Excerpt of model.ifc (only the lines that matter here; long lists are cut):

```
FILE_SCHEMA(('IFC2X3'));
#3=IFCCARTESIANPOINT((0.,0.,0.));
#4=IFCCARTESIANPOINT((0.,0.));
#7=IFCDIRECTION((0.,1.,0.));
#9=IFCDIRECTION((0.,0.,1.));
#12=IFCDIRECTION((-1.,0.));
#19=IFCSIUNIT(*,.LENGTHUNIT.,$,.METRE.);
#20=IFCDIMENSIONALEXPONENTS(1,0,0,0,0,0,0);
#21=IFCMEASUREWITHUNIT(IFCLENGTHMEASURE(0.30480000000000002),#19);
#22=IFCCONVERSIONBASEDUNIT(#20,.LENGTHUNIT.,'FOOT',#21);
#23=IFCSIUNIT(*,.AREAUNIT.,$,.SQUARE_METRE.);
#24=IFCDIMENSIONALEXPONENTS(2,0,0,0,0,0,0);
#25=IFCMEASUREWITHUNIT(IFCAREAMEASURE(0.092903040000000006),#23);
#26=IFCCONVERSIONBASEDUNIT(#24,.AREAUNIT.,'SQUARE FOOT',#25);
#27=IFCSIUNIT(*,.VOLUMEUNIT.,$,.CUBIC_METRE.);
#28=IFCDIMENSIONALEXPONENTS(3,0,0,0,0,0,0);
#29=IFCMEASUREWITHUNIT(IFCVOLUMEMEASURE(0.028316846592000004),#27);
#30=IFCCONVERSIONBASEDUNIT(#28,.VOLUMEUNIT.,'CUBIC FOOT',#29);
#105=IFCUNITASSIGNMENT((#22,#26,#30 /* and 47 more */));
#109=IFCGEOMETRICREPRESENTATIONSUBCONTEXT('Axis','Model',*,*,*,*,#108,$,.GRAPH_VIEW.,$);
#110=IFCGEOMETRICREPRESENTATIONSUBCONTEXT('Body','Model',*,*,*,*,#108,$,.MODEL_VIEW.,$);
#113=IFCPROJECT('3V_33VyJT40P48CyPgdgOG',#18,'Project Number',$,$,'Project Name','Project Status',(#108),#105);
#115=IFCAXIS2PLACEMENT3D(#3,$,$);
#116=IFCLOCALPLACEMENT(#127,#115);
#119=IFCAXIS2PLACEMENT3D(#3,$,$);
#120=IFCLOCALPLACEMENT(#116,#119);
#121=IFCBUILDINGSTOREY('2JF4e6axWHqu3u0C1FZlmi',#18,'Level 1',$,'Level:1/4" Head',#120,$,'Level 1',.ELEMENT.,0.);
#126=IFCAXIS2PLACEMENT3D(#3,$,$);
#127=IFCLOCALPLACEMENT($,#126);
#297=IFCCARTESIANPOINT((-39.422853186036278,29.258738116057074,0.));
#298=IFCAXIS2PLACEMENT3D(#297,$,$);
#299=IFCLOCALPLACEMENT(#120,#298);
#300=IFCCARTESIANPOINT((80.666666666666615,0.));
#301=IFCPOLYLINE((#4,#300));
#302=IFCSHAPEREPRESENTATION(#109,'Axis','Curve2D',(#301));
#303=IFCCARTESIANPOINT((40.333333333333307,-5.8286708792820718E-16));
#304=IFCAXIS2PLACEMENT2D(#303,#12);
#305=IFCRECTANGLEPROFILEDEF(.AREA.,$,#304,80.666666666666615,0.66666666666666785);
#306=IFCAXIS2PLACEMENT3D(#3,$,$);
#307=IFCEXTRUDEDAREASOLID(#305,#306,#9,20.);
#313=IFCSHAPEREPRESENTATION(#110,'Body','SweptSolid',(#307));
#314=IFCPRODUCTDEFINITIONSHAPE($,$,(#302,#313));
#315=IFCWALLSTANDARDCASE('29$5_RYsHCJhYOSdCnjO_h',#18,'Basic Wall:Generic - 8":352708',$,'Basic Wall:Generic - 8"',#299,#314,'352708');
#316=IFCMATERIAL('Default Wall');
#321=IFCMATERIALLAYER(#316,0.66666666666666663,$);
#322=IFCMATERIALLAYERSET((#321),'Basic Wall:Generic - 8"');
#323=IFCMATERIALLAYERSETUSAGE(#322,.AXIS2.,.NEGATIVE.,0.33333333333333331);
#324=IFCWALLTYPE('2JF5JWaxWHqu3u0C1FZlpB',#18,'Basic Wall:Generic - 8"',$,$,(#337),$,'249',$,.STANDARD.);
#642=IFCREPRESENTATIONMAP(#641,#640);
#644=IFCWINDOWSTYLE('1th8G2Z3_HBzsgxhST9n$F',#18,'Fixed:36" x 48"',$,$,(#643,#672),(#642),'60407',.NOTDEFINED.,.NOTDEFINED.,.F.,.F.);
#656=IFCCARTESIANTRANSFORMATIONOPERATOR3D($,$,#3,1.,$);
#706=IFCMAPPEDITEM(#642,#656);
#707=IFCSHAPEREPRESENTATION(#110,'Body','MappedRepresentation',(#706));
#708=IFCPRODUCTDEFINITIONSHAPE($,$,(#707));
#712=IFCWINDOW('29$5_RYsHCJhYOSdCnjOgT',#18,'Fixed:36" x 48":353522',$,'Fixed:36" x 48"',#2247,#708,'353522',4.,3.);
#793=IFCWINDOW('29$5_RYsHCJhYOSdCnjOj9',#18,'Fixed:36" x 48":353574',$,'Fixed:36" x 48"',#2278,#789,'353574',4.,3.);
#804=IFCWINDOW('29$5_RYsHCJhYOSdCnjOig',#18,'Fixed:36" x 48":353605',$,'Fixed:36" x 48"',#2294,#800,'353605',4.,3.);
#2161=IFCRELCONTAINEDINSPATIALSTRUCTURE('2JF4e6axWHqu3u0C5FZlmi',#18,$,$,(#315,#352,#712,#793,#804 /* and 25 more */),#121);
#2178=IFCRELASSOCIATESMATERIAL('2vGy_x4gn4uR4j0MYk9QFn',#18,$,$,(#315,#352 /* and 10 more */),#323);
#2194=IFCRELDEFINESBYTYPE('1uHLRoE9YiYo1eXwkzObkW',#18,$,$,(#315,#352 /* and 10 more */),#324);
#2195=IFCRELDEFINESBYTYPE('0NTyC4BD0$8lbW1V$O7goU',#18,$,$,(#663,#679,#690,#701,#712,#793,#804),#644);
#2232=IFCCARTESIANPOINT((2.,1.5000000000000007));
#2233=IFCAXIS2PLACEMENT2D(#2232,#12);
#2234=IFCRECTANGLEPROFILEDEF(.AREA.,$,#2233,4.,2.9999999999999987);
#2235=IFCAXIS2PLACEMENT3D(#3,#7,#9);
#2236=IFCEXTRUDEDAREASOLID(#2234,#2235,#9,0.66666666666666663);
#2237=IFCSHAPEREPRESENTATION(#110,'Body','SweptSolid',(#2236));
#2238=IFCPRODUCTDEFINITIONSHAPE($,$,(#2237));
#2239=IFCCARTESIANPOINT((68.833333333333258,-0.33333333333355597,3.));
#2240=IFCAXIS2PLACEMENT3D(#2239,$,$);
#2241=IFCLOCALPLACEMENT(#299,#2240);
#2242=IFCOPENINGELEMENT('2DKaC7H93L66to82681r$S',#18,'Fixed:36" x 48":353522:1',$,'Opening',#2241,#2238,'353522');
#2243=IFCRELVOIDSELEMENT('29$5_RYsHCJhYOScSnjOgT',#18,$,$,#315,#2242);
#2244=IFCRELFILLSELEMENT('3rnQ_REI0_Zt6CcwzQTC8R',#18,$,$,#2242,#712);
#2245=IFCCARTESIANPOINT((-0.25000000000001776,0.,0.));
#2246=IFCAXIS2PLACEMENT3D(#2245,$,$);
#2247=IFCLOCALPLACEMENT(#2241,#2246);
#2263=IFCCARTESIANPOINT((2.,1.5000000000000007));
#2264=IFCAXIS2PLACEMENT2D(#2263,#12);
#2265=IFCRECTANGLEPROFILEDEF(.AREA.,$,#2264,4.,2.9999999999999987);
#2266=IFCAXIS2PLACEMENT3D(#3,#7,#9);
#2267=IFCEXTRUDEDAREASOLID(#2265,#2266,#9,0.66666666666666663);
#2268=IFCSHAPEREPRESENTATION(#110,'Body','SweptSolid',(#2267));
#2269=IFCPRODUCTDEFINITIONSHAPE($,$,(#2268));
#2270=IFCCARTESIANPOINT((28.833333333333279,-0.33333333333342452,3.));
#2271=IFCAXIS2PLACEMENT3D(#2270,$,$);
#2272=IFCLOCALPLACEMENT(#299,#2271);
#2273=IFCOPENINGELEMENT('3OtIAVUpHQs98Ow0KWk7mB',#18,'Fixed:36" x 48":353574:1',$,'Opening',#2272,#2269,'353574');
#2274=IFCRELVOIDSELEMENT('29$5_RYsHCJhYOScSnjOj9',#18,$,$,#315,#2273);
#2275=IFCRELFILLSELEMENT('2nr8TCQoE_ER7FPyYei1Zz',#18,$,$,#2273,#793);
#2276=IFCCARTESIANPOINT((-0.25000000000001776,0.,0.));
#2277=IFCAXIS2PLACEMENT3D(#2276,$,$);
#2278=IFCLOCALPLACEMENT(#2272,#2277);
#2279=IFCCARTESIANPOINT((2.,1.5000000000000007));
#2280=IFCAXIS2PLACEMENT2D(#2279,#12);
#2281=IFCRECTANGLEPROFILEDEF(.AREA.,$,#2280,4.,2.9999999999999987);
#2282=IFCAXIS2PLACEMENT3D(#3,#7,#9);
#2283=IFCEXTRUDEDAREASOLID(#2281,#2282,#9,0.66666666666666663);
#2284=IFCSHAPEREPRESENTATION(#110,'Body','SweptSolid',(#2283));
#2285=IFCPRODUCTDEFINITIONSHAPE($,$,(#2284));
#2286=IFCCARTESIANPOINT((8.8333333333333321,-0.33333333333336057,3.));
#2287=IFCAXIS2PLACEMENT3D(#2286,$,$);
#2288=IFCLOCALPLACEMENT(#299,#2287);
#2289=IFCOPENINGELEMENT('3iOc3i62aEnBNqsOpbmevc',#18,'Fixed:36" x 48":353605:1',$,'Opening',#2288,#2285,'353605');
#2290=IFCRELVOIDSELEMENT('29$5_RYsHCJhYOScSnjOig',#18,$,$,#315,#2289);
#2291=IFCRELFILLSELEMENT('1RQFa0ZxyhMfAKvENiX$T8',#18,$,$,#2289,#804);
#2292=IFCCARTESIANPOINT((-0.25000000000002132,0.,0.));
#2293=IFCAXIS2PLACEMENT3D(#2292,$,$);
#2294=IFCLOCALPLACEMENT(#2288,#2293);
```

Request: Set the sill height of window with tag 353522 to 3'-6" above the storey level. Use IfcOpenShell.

```python
import numpy as np
import ifcopenshell
import ifcopenshell.api.geometry
import ifcopenshell.geom
import ifcopenshell.util.element
import ifcopenshell.util.placement
import ifcopenshell.util.shape
import ifcopenshell.util.unit

model = ifcopenshell.open("model.ifc")
unit_scale = ifcopenshell.util.unit.calculate_unit_scale(model)

window = model.by_id(712)
opening = window.FillsVoids[0].RelatingOpeningElement
storey = ifcopenshell.util.element.get_container(window, ifc_class="IfcBuildingStorey")
level = ifcopenshell.util.placement.get_local_placement(storey.ObjectPlacement)[2, 3]

# The opening's origin need not be at the sill, so measure its lowest point.
shape = ifcopenshell.geom.create_shape(ifcopenshell.geom.settings(), opening)
bottom = ifcopenshell.util.shape.get_shape_bottom_elevation(shape, shape.geometry) / unit_scale
dz = level + 42 * 0.0254 / unit_scale - bottom

shift = np.array([0.0, 0.0, dz])
# The window is placed relative to its opening, so it follows when the opening moves.
matrix = ifcopenshell.util.placement.get_local_placement(opening.ObjectPlacement)
matrix[:3, 3] += shift
ifcopenshell.api.geometry.edit_object_placement(
    model, product=opening, matrix=matrix, is_si=False, should_transform_children=True
)

print(f"moved by {dz * unit_scale:+.3f} m")

model.write("model_rev.ifc")
```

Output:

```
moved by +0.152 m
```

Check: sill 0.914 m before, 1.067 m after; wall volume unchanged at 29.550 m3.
